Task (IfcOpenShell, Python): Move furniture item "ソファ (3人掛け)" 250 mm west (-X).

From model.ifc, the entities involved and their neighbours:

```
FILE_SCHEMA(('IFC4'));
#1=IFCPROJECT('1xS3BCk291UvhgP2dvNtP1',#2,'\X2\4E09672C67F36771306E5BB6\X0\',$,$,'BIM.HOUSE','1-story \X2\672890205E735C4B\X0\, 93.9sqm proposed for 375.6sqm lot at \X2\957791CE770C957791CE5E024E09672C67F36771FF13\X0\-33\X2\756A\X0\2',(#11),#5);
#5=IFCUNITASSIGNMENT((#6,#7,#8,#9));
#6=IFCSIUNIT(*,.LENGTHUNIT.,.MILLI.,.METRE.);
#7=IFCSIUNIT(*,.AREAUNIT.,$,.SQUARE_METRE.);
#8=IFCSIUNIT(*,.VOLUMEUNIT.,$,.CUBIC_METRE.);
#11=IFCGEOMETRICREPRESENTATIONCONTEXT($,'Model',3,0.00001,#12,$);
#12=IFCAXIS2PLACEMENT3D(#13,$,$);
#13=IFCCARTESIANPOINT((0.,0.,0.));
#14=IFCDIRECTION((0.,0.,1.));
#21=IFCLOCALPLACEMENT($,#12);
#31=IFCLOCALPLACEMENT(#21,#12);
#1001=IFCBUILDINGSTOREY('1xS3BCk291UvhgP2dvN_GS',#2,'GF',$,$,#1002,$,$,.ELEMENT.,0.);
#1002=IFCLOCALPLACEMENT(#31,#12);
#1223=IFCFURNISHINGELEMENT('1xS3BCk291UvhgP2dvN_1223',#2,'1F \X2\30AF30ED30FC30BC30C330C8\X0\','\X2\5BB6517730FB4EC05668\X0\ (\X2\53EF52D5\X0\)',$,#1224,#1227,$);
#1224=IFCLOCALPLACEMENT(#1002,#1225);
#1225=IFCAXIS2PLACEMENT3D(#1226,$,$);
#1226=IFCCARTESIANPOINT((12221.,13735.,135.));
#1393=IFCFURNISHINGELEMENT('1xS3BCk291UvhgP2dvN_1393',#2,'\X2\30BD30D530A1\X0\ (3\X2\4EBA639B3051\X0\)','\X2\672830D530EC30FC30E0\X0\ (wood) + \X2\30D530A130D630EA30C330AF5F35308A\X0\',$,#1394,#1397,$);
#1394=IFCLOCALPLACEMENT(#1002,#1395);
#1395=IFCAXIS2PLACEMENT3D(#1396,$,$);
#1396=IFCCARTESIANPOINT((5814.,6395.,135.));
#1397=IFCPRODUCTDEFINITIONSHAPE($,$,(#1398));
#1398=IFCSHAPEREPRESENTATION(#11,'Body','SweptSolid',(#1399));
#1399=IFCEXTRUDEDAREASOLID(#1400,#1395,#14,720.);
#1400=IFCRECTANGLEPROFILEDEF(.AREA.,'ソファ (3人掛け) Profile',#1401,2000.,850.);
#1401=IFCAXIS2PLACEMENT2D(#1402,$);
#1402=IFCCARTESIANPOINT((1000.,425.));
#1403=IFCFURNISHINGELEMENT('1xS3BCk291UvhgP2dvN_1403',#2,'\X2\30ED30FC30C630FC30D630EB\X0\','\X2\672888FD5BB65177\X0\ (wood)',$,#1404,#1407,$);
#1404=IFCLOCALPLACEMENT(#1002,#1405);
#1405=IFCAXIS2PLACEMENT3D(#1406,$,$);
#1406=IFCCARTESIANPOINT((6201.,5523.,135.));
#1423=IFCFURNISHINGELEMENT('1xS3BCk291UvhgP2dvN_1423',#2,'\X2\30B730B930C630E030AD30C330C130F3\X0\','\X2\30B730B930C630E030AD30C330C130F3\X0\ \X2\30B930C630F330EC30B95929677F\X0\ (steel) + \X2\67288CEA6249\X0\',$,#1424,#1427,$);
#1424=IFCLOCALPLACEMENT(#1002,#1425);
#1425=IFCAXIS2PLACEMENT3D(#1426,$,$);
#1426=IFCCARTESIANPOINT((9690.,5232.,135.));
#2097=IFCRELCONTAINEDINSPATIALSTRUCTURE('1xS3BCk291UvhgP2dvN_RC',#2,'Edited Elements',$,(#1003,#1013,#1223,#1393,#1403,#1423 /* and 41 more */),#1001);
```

```python
import ifcopenshell
import ifcopenshell.api.geometry
import ifcopenshell.util.placement
import ifcopenshell.util.unit

model = ifcopenshell.open("model.ifc")
unit_scale = ifcopenshell.util.unit.calculate_unit_scale(model)

item = model.by_guid("1xS3BCk291UvhgP2dvN_1393")
matrix = ifcopenshell.util.placement.get_local_placement(item.ObjectPlacement)
matrix[0, 3] -= 0.25 / unit_scale
ifcopenshell.api.geometry.edit_object_placement(model, product=item, matrix=matrix, is_si=False)

print(ifcopenshell.util.placement.get_local_placement(item.ObjectPlacement).round(3) + 0.0)

model.write("model_edited.ifc")
```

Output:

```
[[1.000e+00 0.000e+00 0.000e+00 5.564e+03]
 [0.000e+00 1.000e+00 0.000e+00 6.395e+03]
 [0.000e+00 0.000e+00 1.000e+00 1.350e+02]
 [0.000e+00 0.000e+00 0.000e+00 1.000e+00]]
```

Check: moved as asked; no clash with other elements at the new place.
